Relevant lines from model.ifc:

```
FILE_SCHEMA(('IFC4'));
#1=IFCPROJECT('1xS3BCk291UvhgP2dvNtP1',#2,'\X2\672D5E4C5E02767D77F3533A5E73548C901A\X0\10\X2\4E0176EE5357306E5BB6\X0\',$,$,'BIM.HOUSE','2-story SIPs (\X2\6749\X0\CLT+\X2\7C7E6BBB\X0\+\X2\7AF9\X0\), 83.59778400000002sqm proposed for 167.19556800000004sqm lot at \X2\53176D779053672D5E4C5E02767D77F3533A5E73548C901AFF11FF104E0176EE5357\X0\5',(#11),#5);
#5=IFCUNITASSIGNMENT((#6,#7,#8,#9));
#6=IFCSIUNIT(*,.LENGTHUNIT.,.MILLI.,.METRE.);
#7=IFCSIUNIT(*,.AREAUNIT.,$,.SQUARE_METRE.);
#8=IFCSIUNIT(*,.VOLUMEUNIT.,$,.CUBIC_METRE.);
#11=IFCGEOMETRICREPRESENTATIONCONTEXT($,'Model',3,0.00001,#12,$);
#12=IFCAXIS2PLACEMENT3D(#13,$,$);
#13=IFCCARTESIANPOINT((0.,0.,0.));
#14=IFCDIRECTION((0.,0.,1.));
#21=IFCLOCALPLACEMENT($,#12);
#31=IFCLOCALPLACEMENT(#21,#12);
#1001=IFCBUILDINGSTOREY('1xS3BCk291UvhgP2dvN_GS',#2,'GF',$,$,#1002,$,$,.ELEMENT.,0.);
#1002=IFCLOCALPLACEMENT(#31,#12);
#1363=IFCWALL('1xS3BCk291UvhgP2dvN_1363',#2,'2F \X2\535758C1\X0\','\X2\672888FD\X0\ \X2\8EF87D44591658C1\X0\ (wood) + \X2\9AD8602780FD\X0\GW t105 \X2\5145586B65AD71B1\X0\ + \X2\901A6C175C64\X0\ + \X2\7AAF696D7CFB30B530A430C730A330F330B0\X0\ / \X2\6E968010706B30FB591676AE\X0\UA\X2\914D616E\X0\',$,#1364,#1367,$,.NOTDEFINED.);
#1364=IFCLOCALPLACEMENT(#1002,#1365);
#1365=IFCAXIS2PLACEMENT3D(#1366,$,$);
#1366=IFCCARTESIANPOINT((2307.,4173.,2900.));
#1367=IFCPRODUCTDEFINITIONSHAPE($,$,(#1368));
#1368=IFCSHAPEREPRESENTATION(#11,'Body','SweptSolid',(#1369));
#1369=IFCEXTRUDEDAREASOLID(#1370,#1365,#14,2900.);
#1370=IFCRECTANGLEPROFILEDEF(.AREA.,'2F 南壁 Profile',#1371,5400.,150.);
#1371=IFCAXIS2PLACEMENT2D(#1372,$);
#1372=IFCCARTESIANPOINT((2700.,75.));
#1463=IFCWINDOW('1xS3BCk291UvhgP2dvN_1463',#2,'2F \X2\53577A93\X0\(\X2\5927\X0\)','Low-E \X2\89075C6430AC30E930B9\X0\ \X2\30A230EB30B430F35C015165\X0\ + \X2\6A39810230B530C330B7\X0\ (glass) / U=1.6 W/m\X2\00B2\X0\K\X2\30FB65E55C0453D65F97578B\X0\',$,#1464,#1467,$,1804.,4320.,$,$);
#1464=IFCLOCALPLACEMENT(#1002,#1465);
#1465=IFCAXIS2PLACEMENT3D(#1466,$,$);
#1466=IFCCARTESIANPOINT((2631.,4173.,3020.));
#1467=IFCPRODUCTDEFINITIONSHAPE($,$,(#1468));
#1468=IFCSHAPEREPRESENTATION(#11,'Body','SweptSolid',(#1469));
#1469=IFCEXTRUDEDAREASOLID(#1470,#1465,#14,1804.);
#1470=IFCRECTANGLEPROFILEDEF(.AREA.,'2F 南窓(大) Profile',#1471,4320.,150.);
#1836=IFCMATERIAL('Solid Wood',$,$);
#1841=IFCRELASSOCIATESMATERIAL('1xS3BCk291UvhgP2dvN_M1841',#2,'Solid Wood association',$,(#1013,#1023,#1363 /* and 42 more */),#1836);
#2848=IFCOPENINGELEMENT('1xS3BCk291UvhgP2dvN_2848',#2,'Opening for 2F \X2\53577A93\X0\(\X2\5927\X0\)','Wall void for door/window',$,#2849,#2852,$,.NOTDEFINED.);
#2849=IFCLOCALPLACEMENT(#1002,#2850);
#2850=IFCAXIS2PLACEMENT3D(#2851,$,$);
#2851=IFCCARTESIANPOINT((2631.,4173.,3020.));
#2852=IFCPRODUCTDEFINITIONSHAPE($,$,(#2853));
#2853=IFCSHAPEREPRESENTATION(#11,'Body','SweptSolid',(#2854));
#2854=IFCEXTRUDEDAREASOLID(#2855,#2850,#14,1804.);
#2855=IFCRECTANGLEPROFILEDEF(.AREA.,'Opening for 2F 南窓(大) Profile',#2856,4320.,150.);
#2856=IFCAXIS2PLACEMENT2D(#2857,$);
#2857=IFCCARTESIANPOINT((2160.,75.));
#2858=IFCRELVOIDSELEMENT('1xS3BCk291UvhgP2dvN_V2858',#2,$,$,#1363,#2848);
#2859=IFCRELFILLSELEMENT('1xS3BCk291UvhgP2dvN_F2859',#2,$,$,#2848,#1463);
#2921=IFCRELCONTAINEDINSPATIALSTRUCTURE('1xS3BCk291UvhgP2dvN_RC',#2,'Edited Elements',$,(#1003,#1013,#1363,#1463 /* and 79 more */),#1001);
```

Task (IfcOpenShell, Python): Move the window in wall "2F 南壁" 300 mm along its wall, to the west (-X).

```python
import ifcopenshell
import ifcopenshell.api.geometry
import ifcopenshell.util.placement
import ifcopenshell.util.unit

model = ifcopenshell.open("model.ifc")
unit_scale = ifcopenshell.util.unit.calculate_unit_scale(model)

window = model.by_guid("1xS3BCk291UvhgP2dvN_1463")
opening = window.FillsVoids[0].RelatingOpeningElement
wall = opening.VoidsElements[0].RelatingBuildingElement

wall_matrix = ifcopenshell.util.placement.get_local_placement(wall.ObjectPlacement)
shift = wall_matrix[:3, 0] * -0.3 / unit_scale
before = ifcopenshell.util.placement.get_local_placement(window.ObjectPlacement)[:3, 3].copy()

# The window is not placed relative to its opening, so move both.
for product in (opening, window):
    matrix = ifcopenshell.util.placement.get_local_placement(product.ObjectPlacement)
    matrix[:3, 3] += shift
    ifcopenshell.api.geometry.edit_object_placement(model, product=product, matrix=matrix, is_si=False)

after = ifcopenshell.util.placement.get_local_placement(window.ObjectPlacement)[:3, 3]
print("window moved by", (after - before).round(3) + 0.0)

model.write("model_edited.ifc")
```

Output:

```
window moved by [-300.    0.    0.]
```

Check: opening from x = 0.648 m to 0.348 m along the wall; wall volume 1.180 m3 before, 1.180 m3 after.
